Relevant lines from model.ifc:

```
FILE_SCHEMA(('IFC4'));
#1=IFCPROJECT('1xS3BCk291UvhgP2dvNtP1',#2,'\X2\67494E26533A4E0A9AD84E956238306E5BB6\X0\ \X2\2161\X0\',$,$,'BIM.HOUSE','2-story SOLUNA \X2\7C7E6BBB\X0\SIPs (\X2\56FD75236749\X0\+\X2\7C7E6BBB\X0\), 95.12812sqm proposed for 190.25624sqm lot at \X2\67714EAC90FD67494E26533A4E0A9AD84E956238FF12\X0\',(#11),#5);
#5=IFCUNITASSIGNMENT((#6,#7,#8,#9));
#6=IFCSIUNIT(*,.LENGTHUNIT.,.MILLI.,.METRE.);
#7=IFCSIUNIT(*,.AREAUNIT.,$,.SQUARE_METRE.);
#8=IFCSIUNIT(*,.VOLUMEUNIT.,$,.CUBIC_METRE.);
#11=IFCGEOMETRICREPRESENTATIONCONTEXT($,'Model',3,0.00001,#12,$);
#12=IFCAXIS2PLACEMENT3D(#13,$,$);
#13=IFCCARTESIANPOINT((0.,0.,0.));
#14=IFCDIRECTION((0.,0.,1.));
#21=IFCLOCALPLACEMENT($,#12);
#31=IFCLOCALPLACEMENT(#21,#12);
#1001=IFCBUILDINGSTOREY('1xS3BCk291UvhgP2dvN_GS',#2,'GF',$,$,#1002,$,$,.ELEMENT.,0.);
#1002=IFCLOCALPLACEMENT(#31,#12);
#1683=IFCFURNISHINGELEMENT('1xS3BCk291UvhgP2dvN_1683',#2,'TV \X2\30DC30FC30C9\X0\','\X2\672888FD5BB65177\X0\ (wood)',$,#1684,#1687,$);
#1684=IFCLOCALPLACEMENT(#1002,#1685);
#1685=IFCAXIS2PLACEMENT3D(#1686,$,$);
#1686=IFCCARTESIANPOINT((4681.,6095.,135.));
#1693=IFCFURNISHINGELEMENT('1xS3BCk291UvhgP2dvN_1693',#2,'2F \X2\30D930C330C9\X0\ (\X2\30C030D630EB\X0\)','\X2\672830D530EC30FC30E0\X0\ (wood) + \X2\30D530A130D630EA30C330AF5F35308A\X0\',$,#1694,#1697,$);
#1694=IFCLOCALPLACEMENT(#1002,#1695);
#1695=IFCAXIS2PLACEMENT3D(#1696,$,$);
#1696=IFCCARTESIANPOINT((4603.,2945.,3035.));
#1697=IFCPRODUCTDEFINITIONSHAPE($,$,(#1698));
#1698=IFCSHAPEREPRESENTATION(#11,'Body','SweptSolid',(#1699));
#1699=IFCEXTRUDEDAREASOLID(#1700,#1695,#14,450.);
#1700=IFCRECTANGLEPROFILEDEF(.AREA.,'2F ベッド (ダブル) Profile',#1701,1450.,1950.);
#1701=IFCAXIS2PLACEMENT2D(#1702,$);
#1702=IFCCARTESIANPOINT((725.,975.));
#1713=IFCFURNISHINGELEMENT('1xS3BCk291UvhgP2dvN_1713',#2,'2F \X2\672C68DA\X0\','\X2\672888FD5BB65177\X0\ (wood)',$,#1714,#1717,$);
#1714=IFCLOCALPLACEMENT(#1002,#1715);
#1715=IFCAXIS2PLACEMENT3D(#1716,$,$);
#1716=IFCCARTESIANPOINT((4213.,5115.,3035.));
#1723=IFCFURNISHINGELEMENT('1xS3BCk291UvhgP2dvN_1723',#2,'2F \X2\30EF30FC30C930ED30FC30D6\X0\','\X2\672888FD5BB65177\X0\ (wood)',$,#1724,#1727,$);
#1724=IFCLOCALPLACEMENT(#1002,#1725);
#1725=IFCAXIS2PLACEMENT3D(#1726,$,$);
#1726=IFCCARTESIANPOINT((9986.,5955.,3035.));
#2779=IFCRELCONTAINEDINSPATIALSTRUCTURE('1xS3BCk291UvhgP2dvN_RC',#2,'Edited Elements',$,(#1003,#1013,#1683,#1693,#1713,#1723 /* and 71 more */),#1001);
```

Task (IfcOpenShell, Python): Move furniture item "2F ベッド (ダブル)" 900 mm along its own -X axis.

```python
import ifcopenshell
import ifcopenshell.api.geometry
import ifcopenshell.util.placement
import ifcopenshell.util.unit

model = ifcopenshell.open("model.ifc")
unit_scale = ifcopenshell.util.unit.calculate_unit_scale(model)

item = model.by_guid("1xS3BCk291UvhgP2dvN_1693")
matrix = ifcopenshell.util.placement.get_local_placement(item.ObjectPlacement)
matrix[:3, 3] -= matrix[:3, 0] * 0.9 / unit_scale
ifcopenshell.api.geometry.edit_object_placement(model, product=item, matrix=matrix, is_si=False)

print(ifcopenshell.util.placement.get_local_placement(item.ObjectPlacement).round(3) + 0.0)

model.write("model_edited.ifc")
```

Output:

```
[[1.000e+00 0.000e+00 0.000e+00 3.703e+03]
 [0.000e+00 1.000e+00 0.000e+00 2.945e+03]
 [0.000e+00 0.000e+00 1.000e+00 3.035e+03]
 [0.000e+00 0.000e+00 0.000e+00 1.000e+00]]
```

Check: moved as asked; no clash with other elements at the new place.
